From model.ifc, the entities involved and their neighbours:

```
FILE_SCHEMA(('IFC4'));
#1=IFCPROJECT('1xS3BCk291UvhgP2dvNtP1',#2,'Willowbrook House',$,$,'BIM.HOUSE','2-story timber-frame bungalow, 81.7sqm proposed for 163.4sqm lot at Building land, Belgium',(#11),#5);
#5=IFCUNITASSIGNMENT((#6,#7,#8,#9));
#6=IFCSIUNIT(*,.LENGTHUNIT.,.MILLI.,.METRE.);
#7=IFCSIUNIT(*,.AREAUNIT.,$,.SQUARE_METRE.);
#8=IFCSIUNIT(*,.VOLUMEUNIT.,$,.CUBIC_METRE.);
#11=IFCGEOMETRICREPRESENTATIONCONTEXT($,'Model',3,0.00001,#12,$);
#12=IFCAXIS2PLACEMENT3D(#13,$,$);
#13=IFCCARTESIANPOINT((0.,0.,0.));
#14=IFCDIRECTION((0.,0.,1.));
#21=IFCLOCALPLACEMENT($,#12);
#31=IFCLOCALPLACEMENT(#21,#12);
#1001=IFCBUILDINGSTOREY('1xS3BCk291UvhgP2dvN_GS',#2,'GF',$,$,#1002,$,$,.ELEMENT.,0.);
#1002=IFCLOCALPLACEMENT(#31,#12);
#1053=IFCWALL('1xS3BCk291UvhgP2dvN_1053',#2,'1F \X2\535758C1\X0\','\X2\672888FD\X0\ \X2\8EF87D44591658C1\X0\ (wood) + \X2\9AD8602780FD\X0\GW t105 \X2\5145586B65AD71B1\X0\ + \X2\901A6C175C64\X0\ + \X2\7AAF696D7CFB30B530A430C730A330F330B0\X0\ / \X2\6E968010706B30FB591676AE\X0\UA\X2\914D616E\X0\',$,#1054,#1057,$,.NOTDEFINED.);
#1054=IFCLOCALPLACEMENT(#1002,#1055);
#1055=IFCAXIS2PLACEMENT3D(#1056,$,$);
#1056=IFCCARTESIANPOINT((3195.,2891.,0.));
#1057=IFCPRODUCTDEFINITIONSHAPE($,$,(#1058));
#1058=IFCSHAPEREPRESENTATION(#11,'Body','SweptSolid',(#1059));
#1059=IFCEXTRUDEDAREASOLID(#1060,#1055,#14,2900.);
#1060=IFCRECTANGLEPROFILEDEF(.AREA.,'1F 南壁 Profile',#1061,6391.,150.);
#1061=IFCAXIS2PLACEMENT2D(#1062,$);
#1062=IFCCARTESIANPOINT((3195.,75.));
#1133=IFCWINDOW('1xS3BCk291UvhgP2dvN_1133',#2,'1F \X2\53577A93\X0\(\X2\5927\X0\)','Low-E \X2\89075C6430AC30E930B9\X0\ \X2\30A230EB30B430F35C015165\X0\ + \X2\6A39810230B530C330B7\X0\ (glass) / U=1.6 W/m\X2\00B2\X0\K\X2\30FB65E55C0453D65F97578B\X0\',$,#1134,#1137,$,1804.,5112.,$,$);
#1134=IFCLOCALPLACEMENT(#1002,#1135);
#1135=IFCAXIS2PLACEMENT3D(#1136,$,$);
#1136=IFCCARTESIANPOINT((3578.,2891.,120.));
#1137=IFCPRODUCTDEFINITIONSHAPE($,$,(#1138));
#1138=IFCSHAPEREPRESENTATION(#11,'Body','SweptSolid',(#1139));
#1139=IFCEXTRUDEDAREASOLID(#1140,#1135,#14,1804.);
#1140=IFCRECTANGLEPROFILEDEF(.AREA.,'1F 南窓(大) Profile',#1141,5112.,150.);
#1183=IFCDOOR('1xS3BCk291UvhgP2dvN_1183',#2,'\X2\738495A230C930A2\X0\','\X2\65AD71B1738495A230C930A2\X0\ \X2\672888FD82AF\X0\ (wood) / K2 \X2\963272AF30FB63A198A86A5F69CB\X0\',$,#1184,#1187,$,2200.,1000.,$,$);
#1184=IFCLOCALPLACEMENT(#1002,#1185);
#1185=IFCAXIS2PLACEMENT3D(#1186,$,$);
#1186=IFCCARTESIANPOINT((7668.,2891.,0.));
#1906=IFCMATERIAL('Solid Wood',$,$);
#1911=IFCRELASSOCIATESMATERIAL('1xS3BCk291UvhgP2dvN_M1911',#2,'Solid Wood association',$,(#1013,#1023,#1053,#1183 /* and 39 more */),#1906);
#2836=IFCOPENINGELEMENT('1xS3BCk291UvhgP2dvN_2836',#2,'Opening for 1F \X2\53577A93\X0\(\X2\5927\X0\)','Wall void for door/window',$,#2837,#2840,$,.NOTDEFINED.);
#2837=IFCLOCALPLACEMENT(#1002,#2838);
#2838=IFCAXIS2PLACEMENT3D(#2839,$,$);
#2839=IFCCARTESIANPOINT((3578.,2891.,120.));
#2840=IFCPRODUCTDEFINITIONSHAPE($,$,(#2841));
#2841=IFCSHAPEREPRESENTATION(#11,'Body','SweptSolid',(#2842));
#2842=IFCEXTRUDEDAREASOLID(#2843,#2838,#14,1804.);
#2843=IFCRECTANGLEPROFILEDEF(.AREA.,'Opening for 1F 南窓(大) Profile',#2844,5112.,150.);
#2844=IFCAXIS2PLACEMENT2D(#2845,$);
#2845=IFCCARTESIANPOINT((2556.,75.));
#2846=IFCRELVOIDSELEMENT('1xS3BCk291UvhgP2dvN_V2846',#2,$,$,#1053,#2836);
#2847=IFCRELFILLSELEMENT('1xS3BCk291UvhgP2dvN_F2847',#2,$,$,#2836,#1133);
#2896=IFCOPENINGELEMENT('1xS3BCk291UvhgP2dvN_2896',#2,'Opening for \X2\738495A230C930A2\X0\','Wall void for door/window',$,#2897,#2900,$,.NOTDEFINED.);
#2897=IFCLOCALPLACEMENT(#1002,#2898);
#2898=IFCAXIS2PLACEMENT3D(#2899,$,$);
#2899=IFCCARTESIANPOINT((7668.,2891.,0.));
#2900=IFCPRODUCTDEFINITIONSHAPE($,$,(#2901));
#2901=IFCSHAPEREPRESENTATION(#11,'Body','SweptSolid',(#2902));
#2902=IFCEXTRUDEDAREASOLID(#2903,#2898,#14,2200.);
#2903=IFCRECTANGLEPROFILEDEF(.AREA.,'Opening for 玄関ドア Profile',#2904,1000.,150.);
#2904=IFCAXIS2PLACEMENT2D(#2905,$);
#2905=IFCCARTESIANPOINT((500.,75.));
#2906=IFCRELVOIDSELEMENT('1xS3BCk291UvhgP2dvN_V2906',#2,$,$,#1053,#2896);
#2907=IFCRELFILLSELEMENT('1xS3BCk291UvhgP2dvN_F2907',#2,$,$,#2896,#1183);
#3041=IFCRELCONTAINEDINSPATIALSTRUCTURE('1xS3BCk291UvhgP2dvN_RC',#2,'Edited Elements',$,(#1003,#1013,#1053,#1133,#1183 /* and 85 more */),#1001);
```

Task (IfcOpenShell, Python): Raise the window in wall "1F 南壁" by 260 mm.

```python
import numpy as np
import ifcopenshell
import ifcopenshell.api.geometry
import ifcopenshell.util.placement
import ifcopenshell.util.unit

model = ifcopenshell.open("model.ifc")
unit_scale = ifcopenshell.util.unit.calculate_unit_scale(model)

window = model.by_guid("1xS3BCk291UvhgP2dvN_1133")
opening = window.FillsVoids[0].RelatingOpeningElement
dz = 0.26 / unit_scale

shift = np.array([0.0, 0.0, dz])
# The window is not placed relative to its opening, so move both.
for product in (opening, window):
    matrix = ifcopenshell.util.placement.get_local_placement(product.ObjectPlacement)
    matrix[:3, 3] += shift
    ifcopenshell.api.geometry.edit_object_placement(model, product=product, matrix=matrix, is_si=False)

print(f"moved by {dz * unit_scale:+.3f} m")

model.write("model_edited.ifc")
```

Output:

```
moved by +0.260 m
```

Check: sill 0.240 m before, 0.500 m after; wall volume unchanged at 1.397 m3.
